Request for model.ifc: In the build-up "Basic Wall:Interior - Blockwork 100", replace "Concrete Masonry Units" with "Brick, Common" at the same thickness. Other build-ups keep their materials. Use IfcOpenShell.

First a look at what the model holds.

```python
import ifcopenshell
import ifcopenshell.util.element

model = ifcopenshell.open("model.ifc")
print(model.schema)
for layer_set in model.by_type("IfcMaterialLayerSet"):
    if layer_set.LayerSetName == "Basic Wall:Interior - Blockwork 100":
        for layer in layer_set.MaterialLayers:
            print(layer.id(), layer.Material and layer.Material.Name, layer.LayerThickness, sep=" | ")
        print(len(ifcopenshell.util.element.get_elements_by_material(model, layer_set)), "elements and types use it")
print(sorted(m.Name for m in model.by_type("IfcMaterial") if m.Name)[:60])
```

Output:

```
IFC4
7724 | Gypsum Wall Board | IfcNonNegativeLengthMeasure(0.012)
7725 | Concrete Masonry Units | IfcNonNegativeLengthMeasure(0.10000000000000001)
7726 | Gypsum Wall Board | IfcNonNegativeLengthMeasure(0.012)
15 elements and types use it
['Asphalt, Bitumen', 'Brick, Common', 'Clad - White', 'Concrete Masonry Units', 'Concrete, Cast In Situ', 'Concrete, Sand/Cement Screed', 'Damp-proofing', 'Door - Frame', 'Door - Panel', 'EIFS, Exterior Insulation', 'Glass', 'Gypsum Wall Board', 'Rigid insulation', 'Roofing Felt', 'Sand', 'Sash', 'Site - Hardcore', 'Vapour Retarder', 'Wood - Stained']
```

```python
import ifcopenshell
import ifcopenshell.api.material

model = ifcopenshell.open("model.ifc")

layer_set = next(s for s in model.by_type("IfcMaterialLayerSet") if s.LayerSetName == "Basic Wall:Interior - Blockwork 100")
layer = next(l for l in layer_set.MaterialLayers if l.Material and l.Material.Name == "Concrete Masonry Units")
material = next(m for m in model.by_type("IfcMaterial") if m.Name == "Brick, Common")

# Point this one layer at the other material; renaming the old one would change it everywhere.
ifcopenshell.api.material.edit_layer(model, layer=layer, attributes={"Name": material.Name}, material=material)

print([l.Material.Name if l.Material else None for l in layer_set.MaterialLayers])

model.write("model_v2.ifc")
```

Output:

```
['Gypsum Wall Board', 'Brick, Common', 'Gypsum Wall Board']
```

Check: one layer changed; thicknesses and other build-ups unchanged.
